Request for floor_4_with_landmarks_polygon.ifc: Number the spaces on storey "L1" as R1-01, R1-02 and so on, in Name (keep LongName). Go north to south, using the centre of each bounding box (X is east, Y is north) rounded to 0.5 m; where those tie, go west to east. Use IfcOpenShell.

First a look at what the model holds.

```python
import ifcopenshell
import ifcopenshell.util.element
import ifcopenshell.util.placement

model = ifcopenshell.open("floor_4_with_landmarks_polygon.ifc")
print(model.schema)
storey = next(s for s in model.by_type("IfcBuildingStorey") if s.Name == "L1")
spaces = [e for e in ifcopenshell.util.element.get_decomposition(storey) if e.is_a("IfcSpace")]
for e in sorted(spaces, key=lambda e: e.id()):
    origin = ifcopenshell.util.placement.get_local_placement(e.ObjectPlacement)[:3, 3]
    print(e.id(), e.Name, e.LongName, origin.round(2) + 0.0, sep=" | ")
```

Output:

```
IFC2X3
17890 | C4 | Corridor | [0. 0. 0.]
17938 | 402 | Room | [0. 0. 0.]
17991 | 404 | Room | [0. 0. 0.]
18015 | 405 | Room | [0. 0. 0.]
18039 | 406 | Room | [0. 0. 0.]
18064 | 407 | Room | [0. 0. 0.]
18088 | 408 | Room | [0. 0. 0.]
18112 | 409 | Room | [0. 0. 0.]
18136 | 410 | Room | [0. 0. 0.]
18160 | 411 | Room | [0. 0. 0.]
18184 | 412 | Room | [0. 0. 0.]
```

```python
import ifcopenshell
import ifcopenshell.geom
import ifcopenshell.util.element
import ifcopenshell.util.shape

model = ifcopenshell.open("floor_4_with_landmarks_polygon.ifc")
settings = ifcopenshell.geom.settings()
settings.set("use-world-coords", True)


def centre(element):
    shape = ifcopenshell.geom.create_shape(settings, element)
    return ifcopenshell.util.shape.get_bbox_centroid(shape.geometry)


storey = next(s for s in model.by_type("IfcBuildingStorey") if s.Name == "L1")
spaces = [e for e in ifcopenshell.util.element.get_decomposition(storey) if e.is_a("IfcSpace")]

# Insertion points can sit at a corner or the storey origin, so sort by the geometry (in metres).
centres = {e: centre(e) for e in spaces}
spaces.sort(key=lambda e: (-round(centres[e][1] / 0.5), centres[e][0]))

for i, e in enumerate(spaces, start=1):
    number = f"R1-{i:02d}"
    e.Name = number
    print(e.id(), number)

model.write("floor_4_with_landmarks_polygon_v2.ifc")
```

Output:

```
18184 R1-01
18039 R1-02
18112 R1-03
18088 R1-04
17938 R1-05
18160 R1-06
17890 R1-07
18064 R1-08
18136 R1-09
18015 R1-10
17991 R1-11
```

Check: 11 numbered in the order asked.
